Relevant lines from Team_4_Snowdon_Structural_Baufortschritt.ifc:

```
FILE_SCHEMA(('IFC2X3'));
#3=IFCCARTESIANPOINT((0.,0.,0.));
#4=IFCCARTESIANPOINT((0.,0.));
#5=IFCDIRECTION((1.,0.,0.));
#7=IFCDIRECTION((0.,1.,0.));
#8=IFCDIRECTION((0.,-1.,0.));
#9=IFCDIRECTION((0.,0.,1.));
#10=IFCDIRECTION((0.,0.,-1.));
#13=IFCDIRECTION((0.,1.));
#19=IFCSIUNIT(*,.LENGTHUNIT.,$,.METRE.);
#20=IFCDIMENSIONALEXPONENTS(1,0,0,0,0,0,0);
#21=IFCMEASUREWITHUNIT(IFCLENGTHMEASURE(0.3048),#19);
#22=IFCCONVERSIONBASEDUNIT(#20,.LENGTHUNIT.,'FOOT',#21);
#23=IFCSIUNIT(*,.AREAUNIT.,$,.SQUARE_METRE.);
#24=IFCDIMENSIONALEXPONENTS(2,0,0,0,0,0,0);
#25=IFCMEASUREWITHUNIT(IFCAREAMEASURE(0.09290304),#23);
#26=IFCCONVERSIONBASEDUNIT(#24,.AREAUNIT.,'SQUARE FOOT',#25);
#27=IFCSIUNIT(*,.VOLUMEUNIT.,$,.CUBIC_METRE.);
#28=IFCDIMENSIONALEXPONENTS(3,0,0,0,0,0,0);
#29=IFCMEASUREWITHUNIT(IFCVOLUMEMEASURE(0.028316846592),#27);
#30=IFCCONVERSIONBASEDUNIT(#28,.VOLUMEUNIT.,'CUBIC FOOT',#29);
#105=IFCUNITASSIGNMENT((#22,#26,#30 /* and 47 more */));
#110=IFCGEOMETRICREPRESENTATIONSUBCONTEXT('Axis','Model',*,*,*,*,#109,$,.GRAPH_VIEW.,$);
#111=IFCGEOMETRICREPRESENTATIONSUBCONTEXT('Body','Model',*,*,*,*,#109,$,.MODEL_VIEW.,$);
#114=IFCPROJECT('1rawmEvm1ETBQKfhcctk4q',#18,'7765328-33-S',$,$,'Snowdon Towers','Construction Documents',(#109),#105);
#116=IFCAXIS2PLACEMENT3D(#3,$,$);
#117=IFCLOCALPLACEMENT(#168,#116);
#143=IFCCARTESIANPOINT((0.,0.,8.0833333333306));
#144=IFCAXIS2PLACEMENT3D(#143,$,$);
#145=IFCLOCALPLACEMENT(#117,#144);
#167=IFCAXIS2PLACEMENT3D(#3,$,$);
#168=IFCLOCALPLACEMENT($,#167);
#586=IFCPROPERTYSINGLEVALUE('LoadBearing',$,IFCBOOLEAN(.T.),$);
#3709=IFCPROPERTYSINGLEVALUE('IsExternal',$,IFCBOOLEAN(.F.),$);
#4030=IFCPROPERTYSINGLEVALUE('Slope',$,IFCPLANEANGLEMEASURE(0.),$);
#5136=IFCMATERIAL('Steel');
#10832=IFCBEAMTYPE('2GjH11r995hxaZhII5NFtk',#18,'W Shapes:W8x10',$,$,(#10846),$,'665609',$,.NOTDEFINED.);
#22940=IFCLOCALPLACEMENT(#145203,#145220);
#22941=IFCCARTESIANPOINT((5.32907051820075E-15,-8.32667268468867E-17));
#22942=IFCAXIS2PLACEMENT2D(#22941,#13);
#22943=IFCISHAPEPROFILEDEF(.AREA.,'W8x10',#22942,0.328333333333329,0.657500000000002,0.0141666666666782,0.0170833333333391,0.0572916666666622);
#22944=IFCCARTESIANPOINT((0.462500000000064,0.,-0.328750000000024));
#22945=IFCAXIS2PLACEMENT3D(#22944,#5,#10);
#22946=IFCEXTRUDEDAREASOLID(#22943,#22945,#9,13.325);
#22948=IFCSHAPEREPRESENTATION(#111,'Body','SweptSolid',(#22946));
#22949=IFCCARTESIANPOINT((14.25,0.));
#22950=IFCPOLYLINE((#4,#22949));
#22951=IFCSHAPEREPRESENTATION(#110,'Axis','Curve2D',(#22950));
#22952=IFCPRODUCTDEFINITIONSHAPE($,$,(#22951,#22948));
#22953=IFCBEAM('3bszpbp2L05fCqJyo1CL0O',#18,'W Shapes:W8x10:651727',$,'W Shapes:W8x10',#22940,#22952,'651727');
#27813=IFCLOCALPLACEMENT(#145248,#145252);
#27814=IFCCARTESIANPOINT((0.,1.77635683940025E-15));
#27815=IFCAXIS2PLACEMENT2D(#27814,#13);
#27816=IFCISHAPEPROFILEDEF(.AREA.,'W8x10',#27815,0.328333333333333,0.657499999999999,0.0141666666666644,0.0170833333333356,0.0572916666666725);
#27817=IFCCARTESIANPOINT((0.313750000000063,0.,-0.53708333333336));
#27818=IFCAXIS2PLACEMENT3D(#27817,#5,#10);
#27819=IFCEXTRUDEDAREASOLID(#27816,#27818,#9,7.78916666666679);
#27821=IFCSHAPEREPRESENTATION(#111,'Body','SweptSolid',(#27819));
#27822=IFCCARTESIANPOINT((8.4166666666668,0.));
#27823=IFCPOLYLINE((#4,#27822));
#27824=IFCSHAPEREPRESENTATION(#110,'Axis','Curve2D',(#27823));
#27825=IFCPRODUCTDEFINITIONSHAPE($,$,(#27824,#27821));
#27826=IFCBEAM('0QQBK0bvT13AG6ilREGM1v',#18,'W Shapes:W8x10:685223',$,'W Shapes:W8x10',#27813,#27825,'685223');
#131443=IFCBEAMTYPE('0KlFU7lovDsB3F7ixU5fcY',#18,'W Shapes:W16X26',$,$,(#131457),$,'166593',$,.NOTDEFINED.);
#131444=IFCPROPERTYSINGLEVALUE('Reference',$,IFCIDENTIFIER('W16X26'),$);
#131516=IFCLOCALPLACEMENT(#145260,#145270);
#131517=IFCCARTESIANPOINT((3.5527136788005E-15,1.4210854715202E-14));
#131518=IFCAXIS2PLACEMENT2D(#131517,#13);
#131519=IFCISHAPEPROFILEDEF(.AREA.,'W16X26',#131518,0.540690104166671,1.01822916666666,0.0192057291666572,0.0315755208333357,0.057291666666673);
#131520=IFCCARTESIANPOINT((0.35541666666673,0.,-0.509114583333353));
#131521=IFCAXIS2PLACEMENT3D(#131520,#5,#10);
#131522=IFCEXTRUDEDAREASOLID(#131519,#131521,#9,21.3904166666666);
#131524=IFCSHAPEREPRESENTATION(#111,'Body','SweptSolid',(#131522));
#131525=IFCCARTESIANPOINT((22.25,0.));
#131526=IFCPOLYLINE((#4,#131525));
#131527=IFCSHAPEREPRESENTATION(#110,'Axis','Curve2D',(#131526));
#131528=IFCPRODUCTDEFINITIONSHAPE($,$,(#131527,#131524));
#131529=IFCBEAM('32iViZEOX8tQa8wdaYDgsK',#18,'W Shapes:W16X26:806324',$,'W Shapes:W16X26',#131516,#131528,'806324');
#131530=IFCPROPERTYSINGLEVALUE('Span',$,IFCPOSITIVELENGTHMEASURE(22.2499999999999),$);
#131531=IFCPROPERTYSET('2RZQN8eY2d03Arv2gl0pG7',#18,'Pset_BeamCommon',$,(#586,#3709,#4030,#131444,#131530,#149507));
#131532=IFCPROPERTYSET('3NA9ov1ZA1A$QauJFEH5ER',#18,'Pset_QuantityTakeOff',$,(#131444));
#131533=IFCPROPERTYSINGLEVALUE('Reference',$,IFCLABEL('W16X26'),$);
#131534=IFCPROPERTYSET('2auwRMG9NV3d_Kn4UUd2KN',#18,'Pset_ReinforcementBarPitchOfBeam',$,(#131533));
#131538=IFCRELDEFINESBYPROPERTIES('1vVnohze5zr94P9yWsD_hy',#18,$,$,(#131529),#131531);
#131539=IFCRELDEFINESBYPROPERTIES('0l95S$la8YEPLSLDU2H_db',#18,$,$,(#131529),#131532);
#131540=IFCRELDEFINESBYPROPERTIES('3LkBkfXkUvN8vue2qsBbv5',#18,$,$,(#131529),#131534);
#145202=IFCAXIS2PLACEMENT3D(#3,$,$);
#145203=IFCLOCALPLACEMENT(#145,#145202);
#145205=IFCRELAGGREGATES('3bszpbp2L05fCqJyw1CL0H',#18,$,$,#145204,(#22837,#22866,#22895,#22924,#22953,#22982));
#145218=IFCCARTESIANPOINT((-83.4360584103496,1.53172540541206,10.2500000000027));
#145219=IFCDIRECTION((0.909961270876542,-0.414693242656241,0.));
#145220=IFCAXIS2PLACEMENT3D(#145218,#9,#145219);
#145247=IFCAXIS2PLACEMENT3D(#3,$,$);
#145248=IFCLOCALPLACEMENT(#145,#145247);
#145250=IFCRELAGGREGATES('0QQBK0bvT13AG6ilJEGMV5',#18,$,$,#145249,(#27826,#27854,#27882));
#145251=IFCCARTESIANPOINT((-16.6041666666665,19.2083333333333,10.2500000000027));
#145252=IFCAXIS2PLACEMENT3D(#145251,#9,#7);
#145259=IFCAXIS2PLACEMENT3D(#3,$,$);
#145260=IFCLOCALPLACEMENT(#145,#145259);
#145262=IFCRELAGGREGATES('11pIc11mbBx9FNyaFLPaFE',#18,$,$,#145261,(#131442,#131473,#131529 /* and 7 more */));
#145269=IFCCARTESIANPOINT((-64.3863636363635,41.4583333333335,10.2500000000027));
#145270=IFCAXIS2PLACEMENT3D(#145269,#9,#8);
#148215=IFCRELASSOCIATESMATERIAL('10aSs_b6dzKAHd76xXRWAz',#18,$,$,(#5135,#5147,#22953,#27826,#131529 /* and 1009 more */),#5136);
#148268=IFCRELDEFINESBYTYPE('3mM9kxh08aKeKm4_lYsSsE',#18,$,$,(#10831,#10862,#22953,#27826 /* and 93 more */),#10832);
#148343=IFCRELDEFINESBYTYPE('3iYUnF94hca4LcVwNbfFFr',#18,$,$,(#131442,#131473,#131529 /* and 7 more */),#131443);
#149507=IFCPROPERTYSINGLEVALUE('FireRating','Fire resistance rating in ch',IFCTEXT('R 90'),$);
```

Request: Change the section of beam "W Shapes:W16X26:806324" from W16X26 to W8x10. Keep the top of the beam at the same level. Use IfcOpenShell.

```python
import ifcopenshell
import ifcopenshell.api.pset
import ifcopenshell.api.type
import ifcopenshell.util.element
import ifcopenshell.util.representation

model = ifcopenshell.open("Team_4_Snowdon_Structural_Baufortschritt.ifc")

member = model.by_guid("32iViZEOX8tQa8wdaYDgsK")
source = next(p for p in model.by_type("IfcIShapeProfileDef") if p.ProfileName == "W8x10")

body = ifcopenshell.util.representation.get_representation(member, "Model", "Body")
solid = body.Items[0]
old_profile = solid.SweptArea

# Copy the section's sizes but keep this member's own profile position.
profile = ifcopenshell.util.element.copy(model, source)
# Profiles are centred, so shift by half the change in depth to hold the top.
shift = (old_profile.OverallDepth - profile.OverallDepth) / 2
x, y = old_profile.Position.Location.Coordinates
up = (-1.0, 0.0)  # upwards, in the solid's own plane
location = model.createIfcCartesianPoint((x + up[0] * shift, y + up[1] * shift))
profile.Position = model.createIfcAxis2Placement2D(location, old_profile.Position.RefDirection)
solid.SweptArea = profile
if not model.get_total_inverses(old_profile):
    ifcopenshell.util.element.remove_deep2(model, old_profile)

new_type = model.by_guid("2GjH11r995hxaZhII5NFtk")
ifcopenshell.api.type.assign_type(
    model, related_objects=[member], relating_type=new_type, should_map_representations=False
)
member.Name = member.Name.replace("W16X26", "W8x10")
member.ObjectType = "W Shapes:W8x10"
pset = model.by_id(ifcopenshell.util.element.get_pset(member, "Pset_BeamCommon", should_inherit=False)["id"])
ifcopenshell.api.pset.edit_pset(model, pset=pset, properties={"Reference": "W8x10"})
pset = model.by_id(ifcopenshell.util.element.get_pset(member, "Pset_QuantityTakeOff", should_inherit=False)["id"])
ifcopenshell.api.pset.edit_pset(model, pset=pset, properties={"Reference": "W8x10"})
pset = model.by_id(ifcopenshell.util.element.get_pset(member, "Pset_ReinforcementBarPitchOfBeam", should_inherit=False)["id"])
ifcopenshell.api.pset.edit_pset(model, pset=pset, properties={"Reference": "W8x10"})

print(solid.SweptArea)

model.write("Team_4_Snowdon_Structural_Baufortschritt-out.ifc")
```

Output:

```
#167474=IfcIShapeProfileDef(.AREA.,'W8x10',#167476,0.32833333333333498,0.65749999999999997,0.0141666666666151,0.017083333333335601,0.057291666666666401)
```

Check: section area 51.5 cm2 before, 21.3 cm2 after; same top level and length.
